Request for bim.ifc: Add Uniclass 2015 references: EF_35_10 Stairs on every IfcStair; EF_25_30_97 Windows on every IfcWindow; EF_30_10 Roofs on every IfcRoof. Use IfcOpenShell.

First a look at what the model holds.

```python
import ifcopenshell

model = ifcopenshell.open("bim.ifc")
print(model.schema)
print("classifications:", [c.Name for c in model.by_type("IfcClassification")])
for ifc_class in ("IfcDoor", "IfcRoof", "IfcStair", "IfcWall", "IfcWindow"):
    print(ifc_class, len(model.by_type(ifc_class)))
```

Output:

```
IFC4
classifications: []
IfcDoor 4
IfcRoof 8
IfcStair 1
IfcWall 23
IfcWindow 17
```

```python
import ifcopenshell
import ifcopenshell.api.classification

model = ifcopenshell.open("bim.ifc")

system = ifcopenshell.api.classification.add_classification(model, classification="Uniclass 2015")

codes = {
    "IfcStair": ("EF_35_10", "Stairs"),
    "IfcWindow": ("EF_25_30_97", "Windows"),
    "IfcRoof": ("EF_30_10", "Roofs"),
}
for ifc_class, (code, name) in codes.items():
    products = model.by_type(ifc_class)
    ifcopenshell.api.classification.add_reference(
        model, products=products, classification=system, identification=code, name=name
    )
    print(code, len(products))

model.write("bim_updated.ifc")
```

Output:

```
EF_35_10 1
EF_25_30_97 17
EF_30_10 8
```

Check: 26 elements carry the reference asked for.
